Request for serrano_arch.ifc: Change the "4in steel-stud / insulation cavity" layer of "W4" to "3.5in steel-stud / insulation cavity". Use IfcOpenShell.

First a look at what the model holds.

```python
import ifcopenshell
import ifcopenshell.util.element

model = ifcopenshell.open("serrano_arch.ifc")
print(model.schema)
for layer_set in model.by_type("IfcMaterialLayerSet"):
    if layer_set.LayerSetName == "W4":
        for layer in layer_set.MaterialLayers:
            print(layer.id(), layer.Material and layer.Material.Name, layer.LayerThickness, sep=" | ")
        print(len(ifcopenshell.util.element.get_elements_by_material(model, layer_set)), "elements and types use it")
print(sorted(m.Name for m in model.by_type("IfcMaterial") if m.Name)[:60])
```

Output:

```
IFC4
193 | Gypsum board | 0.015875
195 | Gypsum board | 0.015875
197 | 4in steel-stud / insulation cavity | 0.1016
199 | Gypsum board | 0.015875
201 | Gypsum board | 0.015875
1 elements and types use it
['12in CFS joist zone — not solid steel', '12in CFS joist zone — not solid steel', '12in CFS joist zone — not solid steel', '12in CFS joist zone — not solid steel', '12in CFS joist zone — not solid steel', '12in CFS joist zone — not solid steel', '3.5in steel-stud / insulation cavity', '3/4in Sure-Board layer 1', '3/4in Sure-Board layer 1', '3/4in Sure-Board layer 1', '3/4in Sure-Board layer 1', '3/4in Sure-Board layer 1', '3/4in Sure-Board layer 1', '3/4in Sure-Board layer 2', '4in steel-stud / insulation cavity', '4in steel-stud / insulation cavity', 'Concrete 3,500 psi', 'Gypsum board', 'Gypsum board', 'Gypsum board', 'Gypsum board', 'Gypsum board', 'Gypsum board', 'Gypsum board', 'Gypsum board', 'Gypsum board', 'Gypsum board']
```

```python
import ifcopenshell
import ifcopenshell.api.material

model = ifcopenshell.open("serrano_arch.ifc")

layer_set = next(s for s in model.by_type("IfcMaterialLayerSet") if s.LayerSetName == "W4")
layer = next(l for l in layer_set.MaterialLayers if l.Material and l.Material.Name == "4in steel-stud / insulation cavity")
material = next(m for m in model.by_type("IfcMaterial") if m.Name == "3.5in steel-stud / insulation cavity")

# Point this one layer at the other material; renaming the old one would change it everywhere.
ifcopenshell.api.material.edit_layer(model, layer=layer, attributes={}, material=material)

print([l.Material.Name if l.Material else None for l in layer_set.MaterialLayers])

model.write("serrano_arch-out.ifc")
```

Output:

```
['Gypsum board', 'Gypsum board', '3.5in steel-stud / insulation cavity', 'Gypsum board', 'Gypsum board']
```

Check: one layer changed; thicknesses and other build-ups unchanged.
